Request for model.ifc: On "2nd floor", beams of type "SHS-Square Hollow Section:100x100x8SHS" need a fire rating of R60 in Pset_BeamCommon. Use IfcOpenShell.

First a look at what the model holds.

```python
import ifcopenshell
import ifcopenshell.util.element

model = ifcopenshell.open("model.ifc")
print(model.schema)
storey = next(s for s in model.by_type("IfcBuildingStorey") if s.Name == "2nd floor")
beams = [e for e in ifcopenshell.util.element.get_decomposition(storey) if e.is_a("IfcBeam")]
seen = {}
for e in beams:
    element_type = ifcopenshell.util.element.get_type(e)
    key = (element_type.Name if element_type != e and element_type else None, ifcopenshell.util.element.get_pset(e, "Pset_BeamCommon", "FireRating"))
    seen[key] = seen.get(key, 0) + 1
for (name, value), count in sorted(seen.items(), key=str):
    print(count, "x", name, "|", value)
```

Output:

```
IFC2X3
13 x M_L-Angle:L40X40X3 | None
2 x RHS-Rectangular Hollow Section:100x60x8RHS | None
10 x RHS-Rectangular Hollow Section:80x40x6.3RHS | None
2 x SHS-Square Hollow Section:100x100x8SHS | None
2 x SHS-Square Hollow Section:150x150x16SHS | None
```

```python
import ifcopenshell
import ifcopenshell.api.pset
import ifcopenshell.util.element

model = ifcopenshell.open("model.ifc")

storey = next(s for s in model.by_type("IfcBuildingStorey") if s.Name == "2nd floor")
beams = [e for e in ifcopenshell.util.element.get_decomposition(storey) if e.is_a("IfcBeam")]

count = 0
for e in beams:
    element_type = ifcopenshell.util.element.get_type(e)
    if element_type in (None, e) or element_type.Name != "SHS-Square Hollow Section:100x100x8SHS":
        continue
    # add_pset returns the element's existing set when there is one.
    pset = ifcopenshell.api.pset.add_pset(model, product=e, name="Pset_BeamCommon")
    ifcopenshell.api.pset.edit_pset(model, pset=pset, properties={"FireRating": "R60"})
    count += 1

print(count, "beams updated")

model.write("model_rev.ifc")
```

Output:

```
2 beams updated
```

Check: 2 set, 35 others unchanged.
